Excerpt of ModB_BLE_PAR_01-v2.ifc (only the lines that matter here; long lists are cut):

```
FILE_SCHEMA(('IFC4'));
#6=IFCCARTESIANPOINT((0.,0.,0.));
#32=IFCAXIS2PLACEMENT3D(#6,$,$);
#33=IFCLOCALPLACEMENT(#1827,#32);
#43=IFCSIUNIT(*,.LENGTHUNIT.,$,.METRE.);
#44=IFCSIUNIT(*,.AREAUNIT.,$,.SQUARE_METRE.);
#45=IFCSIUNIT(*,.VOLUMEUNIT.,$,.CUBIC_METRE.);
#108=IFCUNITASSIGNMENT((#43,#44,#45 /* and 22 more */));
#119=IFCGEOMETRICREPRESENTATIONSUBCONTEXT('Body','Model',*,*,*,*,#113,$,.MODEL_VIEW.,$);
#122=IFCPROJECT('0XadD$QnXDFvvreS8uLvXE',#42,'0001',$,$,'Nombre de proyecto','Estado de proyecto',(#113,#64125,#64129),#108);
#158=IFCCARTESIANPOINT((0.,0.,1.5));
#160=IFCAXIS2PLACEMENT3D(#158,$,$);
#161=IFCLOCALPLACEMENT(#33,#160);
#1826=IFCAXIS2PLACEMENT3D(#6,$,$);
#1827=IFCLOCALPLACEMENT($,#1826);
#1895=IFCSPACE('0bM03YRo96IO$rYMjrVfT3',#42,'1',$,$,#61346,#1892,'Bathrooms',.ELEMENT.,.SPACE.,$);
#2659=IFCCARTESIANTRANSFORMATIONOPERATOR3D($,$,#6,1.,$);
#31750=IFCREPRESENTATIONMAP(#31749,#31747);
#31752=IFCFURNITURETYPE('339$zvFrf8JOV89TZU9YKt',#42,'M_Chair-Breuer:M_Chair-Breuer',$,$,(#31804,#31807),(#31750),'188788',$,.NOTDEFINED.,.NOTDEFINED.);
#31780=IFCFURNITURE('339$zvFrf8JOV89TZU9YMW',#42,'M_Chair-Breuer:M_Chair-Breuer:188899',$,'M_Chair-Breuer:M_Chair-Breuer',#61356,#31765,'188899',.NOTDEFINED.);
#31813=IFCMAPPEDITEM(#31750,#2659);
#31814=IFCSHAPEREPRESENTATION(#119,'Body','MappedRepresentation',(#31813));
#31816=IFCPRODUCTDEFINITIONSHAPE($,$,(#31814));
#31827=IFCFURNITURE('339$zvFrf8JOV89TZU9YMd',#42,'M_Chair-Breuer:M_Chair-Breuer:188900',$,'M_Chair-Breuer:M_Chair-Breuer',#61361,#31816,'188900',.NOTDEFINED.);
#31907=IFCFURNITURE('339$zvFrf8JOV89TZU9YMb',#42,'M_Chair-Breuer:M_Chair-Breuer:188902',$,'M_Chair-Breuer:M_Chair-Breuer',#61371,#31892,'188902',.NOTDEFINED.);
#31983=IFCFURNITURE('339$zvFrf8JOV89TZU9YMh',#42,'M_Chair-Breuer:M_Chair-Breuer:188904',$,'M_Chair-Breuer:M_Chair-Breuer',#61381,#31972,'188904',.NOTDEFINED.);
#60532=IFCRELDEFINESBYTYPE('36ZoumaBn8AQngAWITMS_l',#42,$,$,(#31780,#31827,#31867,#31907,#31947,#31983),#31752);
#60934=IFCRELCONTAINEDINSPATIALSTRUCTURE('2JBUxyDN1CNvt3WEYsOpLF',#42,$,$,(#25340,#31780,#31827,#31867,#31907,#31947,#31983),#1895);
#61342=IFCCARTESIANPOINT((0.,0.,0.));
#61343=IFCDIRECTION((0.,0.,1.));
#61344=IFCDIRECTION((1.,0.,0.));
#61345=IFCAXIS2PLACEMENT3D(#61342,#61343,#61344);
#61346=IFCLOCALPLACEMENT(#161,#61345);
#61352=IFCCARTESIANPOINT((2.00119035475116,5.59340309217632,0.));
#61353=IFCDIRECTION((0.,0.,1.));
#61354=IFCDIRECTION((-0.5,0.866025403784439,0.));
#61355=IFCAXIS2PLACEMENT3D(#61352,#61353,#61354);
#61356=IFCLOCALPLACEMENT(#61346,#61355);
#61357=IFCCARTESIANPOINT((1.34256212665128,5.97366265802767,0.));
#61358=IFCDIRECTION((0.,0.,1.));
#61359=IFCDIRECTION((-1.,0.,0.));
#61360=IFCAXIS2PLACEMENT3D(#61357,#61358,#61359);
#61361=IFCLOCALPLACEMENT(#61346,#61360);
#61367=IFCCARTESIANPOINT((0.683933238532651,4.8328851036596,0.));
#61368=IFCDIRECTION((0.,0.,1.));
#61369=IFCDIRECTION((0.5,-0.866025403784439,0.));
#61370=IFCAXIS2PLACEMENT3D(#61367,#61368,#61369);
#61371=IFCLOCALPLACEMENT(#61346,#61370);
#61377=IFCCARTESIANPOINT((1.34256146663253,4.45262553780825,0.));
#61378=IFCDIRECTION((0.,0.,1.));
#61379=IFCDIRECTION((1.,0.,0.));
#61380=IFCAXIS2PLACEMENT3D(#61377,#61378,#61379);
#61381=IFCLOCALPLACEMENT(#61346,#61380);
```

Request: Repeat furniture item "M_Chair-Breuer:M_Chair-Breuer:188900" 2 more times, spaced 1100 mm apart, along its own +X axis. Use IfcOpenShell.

```python
import ifcopenshell
import ifcopenshell.api.geometry
import ifcopenshell.api.root
import ifcopenshell.util.element
import ifcopenshell.util.placement
import ifcopenshell.util.unit

model = ifcopenshell.open("ModB_BLE_PAR_01-v2.ifc")
unit_scale = ifcopenshell.util.unit.calculate_unit_scale(model)


def reuse_history(source, copy):
    """copy_class also copies each property set's owner history, people and application; keep the originals."""
    for rel in copy.IsDefinedBy:
        if rel.is_a("IfcRelDefinesByProperties") and (history := rel.RelatingPropertyDefinition.OwnerHistory):
            rel.RelatingPropertyDefinition.OwnerHistory = source.OwnerHistory
            ifcopenshell.util.element.remove_deep2(model, history)


source = model.by_guid("339$zvFrf8JOV89TZU9YMd")
base = ifcopenshell.util.placement.get_local_placement(source.ObjectPlacement)
step = base[:3, 0] * 1.1 / unit_scale

for i in range(1, 3):
    copy = ifcopenshell.api.root.copy_class(model, product=source)
    copy.Representation = ifcopenshell.util.element.copy_deep(
        model, source.Representation, exclude=["IfcGeometricRepresentationContext", "IfcRepresentationMap"]
    )
    copy.Name = "M_Chair-Breuer:M_Chair-Breuer"
    copy.Tag = None
    reuse_history(source, copy)
    matrix = base.copy()
    matrix[:3, 3] += i * step
    print("added at", matrix[:3, 3].round(3) + 0.0)
    ifcopenshell.api.geometry.edit_object_placement(model, product=copy, matrix=matrix, is_si=False)

model.write("ModB_BLE_PAR_01-v2_edited.ifc")
```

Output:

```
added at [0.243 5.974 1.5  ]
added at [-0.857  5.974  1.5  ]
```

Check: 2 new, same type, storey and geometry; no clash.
